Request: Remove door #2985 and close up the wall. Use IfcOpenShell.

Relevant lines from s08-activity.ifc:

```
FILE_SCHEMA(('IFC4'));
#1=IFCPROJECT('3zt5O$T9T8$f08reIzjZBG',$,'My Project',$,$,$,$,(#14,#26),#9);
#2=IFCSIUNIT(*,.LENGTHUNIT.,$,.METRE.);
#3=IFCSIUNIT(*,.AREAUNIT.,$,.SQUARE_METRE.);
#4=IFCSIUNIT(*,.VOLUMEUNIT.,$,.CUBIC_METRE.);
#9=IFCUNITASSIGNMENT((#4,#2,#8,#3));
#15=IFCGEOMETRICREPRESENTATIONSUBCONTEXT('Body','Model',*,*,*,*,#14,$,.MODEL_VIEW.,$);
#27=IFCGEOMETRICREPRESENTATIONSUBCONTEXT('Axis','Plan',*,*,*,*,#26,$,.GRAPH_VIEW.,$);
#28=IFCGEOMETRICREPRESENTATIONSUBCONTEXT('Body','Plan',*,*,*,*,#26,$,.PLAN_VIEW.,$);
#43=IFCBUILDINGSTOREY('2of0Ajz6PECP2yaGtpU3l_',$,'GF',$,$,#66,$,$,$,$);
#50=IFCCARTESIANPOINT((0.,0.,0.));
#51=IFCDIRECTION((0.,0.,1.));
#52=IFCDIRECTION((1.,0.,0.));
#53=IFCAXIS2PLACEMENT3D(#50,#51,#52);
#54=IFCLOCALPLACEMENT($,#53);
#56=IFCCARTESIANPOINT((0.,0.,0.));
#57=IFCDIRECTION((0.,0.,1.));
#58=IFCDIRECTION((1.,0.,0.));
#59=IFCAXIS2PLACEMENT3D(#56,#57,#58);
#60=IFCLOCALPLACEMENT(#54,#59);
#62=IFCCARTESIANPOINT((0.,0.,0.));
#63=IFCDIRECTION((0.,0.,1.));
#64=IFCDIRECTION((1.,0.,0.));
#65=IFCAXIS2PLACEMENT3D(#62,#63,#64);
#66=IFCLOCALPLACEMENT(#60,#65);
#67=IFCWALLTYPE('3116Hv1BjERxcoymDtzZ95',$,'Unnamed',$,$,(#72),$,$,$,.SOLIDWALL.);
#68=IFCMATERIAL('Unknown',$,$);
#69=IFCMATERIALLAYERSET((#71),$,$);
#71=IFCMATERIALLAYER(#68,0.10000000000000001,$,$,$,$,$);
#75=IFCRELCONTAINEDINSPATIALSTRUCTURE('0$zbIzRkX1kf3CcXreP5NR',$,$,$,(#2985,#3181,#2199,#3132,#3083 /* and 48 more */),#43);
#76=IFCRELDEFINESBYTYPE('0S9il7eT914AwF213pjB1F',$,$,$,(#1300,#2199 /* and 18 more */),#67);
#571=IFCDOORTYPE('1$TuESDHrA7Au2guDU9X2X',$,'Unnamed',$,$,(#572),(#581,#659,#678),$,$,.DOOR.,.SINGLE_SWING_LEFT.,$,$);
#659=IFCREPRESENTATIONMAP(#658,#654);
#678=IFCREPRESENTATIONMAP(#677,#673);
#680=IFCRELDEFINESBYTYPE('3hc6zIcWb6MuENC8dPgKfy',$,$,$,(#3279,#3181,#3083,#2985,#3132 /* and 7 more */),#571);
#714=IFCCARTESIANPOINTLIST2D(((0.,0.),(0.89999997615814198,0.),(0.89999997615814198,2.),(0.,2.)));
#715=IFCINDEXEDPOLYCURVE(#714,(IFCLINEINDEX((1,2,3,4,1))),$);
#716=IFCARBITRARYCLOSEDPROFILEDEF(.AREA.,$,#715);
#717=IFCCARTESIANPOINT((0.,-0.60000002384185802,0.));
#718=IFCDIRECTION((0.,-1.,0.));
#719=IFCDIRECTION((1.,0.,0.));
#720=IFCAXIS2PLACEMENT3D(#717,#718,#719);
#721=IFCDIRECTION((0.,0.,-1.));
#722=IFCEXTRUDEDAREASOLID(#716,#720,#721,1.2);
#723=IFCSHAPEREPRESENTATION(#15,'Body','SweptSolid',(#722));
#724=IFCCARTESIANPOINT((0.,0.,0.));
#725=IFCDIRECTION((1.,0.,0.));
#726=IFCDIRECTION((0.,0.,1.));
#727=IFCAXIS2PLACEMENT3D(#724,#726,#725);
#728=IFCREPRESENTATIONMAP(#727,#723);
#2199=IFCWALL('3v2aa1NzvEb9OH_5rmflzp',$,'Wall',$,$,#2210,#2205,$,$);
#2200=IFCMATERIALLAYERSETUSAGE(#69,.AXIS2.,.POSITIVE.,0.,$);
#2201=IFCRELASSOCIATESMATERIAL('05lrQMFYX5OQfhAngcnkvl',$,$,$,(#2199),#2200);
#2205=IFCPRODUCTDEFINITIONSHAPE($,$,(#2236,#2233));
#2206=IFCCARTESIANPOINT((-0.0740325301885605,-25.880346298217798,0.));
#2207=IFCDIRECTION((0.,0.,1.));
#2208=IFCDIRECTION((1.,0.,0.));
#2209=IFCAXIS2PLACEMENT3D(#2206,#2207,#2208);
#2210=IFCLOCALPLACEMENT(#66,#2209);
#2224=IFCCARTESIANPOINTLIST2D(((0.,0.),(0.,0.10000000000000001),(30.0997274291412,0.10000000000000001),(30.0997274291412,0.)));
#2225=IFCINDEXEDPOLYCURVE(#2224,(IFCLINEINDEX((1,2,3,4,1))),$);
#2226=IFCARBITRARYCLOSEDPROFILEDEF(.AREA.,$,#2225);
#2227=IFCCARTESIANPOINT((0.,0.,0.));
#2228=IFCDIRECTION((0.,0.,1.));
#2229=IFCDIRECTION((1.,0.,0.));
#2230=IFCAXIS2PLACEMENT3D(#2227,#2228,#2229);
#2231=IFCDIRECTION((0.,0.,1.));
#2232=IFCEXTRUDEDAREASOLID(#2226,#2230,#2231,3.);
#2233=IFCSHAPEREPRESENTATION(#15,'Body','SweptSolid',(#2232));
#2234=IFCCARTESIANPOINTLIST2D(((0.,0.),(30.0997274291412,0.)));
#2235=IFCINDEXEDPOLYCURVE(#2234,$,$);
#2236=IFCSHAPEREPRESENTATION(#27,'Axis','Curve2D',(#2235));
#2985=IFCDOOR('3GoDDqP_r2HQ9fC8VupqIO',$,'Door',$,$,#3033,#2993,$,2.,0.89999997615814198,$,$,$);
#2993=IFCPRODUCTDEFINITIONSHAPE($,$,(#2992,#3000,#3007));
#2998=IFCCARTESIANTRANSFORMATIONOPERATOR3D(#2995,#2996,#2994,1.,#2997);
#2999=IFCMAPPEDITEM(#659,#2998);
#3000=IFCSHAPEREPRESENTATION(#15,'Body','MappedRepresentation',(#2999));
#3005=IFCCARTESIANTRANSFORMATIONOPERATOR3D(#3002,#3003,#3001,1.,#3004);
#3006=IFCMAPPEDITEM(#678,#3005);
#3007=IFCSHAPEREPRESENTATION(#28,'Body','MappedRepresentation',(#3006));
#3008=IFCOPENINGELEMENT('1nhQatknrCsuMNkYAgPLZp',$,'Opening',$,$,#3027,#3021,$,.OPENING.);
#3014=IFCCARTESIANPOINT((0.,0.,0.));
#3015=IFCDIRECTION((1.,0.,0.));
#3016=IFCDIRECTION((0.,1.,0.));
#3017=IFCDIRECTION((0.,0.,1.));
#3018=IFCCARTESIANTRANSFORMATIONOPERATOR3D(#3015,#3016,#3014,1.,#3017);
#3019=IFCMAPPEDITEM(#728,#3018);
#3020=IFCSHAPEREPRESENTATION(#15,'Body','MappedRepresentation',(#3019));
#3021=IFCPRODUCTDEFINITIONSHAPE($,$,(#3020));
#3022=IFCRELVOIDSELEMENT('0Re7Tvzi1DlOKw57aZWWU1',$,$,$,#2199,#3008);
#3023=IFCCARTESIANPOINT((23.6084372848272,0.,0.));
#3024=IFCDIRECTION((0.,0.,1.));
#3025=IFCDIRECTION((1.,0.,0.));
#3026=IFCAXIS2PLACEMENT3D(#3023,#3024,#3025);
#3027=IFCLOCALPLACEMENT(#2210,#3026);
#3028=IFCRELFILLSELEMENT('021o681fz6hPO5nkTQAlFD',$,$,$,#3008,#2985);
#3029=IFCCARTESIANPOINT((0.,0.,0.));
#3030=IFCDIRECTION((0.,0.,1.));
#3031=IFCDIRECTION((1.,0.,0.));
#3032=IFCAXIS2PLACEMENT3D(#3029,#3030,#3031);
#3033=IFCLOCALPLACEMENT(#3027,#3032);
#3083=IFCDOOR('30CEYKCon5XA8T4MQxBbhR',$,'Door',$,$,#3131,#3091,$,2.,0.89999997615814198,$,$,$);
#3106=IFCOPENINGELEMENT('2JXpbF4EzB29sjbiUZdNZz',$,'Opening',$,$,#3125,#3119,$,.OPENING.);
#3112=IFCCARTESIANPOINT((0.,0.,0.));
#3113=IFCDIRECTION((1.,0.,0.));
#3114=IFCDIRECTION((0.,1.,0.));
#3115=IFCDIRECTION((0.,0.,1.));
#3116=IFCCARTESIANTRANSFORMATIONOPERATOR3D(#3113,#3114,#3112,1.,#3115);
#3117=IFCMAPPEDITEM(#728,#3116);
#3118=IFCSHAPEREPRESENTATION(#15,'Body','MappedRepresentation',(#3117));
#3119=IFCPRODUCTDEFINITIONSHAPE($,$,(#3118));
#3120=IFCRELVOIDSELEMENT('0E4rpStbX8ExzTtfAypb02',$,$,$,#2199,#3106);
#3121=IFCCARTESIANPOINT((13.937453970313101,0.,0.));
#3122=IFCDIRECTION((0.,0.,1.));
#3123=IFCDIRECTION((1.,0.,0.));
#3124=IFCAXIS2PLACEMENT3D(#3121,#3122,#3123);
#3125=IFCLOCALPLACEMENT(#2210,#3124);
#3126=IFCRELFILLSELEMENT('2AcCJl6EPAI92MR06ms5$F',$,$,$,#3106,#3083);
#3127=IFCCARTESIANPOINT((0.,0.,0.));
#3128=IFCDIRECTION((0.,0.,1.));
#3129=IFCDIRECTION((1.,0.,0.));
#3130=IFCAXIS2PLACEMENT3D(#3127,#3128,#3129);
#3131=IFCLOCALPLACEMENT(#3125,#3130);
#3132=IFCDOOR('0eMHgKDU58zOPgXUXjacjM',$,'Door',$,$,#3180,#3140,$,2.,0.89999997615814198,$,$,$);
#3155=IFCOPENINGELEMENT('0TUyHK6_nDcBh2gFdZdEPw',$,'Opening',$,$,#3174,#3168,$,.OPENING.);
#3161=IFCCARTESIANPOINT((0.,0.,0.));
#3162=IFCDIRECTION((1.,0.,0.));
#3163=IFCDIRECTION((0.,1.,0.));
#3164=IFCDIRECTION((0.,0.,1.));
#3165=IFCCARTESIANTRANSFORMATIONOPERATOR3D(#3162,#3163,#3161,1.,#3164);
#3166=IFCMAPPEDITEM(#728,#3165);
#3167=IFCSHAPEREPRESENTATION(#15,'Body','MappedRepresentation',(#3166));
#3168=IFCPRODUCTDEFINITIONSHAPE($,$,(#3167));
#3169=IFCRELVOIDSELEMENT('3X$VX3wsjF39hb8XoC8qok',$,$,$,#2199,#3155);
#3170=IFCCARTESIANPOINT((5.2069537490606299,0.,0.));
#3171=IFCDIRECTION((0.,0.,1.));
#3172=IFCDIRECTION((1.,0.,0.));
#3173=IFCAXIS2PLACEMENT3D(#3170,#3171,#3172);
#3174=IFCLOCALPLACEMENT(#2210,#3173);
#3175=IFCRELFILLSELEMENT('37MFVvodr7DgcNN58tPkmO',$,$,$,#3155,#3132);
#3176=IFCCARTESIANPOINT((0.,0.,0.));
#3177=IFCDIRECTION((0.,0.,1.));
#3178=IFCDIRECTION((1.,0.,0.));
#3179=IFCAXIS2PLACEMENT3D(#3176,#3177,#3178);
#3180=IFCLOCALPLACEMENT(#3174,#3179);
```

```python
import ifcopenshell
import ifcopenshell.api.feature
import ifcopenshell.api.root
import ifcopenshell.geom
import ifcopenshell.util.shape

model = ifcopenshell.open("s08-activity.ifc")
settings = ifcopenshell.geom.settings()


def volume(element):
    """Net volume in cubic metres, openings subtracted."""
    shape = ifcopenshell.geom.create_shape(settings, element)
    return ifcopenshell.util.shape.get_volume(shape.geometry)


door = model.by_guid("3GoDDqP_r2HQ9fC8VupqIO")
opening = door.FillsVoids[0].RelatingOpeningElement
wall = opening.VoidsElements[0].RelatingBuildingElement
before = volume(wall)

ifcopenshell.api.root.remove_product(model, product=door)
ifcopenshell.api.feature.remove_feature(model, feature=opening)

after = volume(wall)

print(f"wall volume {before:.3f} -> {after:.3f} m3")

model.write("s08-activity_v2.ifc")
```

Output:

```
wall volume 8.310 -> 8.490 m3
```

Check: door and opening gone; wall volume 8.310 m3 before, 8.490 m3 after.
